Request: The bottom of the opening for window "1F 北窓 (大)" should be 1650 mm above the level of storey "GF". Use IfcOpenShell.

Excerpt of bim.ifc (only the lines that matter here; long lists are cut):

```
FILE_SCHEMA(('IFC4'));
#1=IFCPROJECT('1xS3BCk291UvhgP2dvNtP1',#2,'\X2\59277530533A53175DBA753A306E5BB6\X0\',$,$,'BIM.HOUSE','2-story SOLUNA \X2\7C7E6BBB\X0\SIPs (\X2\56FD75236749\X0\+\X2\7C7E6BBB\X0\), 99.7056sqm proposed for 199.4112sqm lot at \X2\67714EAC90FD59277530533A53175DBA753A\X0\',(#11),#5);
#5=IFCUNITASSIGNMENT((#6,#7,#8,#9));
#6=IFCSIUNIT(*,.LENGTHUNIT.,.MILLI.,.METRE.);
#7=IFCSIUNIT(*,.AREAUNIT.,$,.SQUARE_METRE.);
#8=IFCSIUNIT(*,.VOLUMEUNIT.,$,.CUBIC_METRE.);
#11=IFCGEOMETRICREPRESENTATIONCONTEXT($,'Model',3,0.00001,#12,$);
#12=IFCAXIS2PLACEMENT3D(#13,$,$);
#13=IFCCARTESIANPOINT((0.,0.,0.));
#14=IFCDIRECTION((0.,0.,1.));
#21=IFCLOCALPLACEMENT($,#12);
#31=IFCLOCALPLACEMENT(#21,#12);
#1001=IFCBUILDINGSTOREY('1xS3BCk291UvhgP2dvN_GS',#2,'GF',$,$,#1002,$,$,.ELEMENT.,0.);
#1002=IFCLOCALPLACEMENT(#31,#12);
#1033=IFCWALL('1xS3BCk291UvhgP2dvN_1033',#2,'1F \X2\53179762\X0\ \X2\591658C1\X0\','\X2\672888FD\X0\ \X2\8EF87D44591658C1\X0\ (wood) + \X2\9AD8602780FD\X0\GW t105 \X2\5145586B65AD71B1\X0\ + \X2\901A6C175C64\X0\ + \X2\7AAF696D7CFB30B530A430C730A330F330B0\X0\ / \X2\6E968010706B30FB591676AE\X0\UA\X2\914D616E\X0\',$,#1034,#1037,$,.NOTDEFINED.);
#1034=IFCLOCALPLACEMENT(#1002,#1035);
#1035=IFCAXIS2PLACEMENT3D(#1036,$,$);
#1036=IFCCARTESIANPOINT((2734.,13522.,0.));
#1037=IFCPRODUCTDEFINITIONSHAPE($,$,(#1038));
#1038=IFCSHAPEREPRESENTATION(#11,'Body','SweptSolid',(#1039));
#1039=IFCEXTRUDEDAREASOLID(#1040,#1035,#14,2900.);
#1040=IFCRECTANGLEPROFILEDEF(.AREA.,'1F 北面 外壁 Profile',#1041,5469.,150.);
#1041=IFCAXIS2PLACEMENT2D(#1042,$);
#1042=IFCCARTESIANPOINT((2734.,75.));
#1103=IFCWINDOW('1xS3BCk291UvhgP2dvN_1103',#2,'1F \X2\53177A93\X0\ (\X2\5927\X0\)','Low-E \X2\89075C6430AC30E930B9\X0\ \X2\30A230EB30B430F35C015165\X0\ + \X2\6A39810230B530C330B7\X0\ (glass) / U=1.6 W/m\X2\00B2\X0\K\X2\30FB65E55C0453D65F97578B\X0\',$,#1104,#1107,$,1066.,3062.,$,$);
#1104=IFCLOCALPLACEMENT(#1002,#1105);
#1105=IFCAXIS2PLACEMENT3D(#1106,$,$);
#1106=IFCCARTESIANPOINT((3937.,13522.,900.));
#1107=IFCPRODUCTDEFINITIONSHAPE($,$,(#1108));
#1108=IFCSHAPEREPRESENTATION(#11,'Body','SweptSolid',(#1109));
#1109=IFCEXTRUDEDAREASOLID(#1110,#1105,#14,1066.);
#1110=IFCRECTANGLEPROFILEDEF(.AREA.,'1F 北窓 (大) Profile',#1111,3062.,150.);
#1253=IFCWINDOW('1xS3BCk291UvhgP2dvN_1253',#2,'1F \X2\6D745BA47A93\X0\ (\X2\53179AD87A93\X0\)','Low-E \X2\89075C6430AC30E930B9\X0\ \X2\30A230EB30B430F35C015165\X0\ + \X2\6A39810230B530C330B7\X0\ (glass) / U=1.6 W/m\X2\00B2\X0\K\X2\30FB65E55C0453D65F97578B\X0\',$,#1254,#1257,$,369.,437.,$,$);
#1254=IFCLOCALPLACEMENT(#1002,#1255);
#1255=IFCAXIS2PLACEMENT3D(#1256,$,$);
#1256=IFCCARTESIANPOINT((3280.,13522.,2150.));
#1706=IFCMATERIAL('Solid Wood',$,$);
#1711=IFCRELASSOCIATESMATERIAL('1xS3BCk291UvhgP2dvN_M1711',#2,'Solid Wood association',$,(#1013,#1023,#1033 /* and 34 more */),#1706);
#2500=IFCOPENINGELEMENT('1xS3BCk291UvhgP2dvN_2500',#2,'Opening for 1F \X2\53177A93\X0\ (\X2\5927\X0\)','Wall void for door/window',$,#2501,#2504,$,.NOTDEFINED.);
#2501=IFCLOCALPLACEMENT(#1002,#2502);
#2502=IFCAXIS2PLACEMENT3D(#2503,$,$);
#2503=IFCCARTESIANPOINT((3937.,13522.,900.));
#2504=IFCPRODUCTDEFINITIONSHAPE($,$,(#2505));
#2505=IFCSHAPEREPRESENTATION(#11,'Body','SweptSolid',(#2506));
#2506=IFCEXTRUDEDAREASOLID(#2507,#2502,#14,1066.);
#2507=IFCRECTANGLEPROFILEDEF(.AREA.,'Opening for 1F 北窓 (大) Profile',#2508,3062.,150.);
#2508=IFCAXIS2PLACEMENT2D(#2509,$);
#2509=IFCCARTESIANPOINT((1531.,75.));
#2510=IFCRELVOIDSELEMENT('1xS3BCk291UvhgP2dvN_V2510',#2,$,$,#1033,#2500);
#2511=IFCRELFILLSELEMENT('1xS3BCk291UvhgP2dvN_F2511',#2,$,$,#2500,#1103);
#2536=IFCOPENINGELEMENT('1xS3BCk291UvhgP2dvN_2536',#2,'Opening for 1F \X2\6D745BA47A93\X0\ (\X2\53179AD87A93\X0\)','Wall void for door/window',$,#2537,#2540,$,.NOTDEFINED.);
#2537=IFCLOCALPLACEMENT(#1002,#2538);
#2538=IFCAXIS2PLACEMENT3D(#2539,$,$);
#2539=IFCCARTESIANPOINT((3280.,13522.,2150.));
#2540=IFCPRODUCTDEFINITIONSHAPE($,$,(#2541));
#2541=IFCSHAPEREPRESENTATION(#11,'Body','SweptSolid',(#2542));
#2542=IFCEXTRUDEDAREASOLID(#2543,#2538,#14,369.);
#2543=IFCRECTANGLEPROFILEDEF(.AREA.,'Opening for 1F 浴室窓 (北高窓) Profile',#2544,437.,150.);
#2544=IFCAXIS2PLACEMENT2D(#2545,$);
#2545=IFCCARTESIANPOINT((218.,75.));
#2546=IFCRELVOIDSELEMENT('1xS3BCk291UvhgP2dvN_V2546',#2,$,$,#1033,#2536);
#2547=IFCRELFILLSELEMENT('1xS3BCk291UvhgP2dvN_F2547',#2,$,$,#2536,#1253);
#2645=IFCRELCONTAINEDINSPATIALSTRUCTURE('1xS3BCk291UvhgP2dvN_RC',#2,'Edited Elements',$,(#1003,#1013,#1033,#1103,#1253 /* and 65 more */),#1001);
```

```python
import numpy as np
import ifcopenshell
import ifcopenshell.api.geometry
import ifcopenshell.geom
import ifcopenshell.util.element
import ifcopenshell.util.placement
import ifcopenshell.util.shape
import ifcopenshell.util.unit

model = ifcopenshell.open("bim.ifc")
unit_scale = ifcopenshell.util.unit.calculate_unit_scale(model)

window = model.by_id(1103)
opening = window.FillsVoids[0].RelatingOpeningElement
storey = ifcopenshell.util.element.get_container(window, ifc_class="IfcBuildingStorey")
level = ifcopenshell.util.placement.get_local_placement(storey.ObjectPlacement)[2, 3]

# The opening's origin need not be at the sill, so measure its lowest point.
shape = ifcopenshell.geom.create_shape(ifcopenshell.geom.settings(), opening)
bottom = ifcopenshell.util.shape.get_shape_bottom_elevation(shape, shape.geometry) / unit_scale
dz = level + 1.65 / unit_scale - bottom

shift = np.array([0.0, 0.0, dz])
# The window is not placed relative to its opening, so move both.
for product in (opening, window):
    matrix = ifcopenshell.util.placement.get_local_placement(product.ObjectPlacement)
    matrix[:3, 3] += shift
    ifcopenshell.api.geometry.edit_object_placement(model, product=product, matrix=matrix, is_si=False)

print(f"moved by {dz * unit_scale:+.3f} m")

model.write("bim_edited.ifc")
```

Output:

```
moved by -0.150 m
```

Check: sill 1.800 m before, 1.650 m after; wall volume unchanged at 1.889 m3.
